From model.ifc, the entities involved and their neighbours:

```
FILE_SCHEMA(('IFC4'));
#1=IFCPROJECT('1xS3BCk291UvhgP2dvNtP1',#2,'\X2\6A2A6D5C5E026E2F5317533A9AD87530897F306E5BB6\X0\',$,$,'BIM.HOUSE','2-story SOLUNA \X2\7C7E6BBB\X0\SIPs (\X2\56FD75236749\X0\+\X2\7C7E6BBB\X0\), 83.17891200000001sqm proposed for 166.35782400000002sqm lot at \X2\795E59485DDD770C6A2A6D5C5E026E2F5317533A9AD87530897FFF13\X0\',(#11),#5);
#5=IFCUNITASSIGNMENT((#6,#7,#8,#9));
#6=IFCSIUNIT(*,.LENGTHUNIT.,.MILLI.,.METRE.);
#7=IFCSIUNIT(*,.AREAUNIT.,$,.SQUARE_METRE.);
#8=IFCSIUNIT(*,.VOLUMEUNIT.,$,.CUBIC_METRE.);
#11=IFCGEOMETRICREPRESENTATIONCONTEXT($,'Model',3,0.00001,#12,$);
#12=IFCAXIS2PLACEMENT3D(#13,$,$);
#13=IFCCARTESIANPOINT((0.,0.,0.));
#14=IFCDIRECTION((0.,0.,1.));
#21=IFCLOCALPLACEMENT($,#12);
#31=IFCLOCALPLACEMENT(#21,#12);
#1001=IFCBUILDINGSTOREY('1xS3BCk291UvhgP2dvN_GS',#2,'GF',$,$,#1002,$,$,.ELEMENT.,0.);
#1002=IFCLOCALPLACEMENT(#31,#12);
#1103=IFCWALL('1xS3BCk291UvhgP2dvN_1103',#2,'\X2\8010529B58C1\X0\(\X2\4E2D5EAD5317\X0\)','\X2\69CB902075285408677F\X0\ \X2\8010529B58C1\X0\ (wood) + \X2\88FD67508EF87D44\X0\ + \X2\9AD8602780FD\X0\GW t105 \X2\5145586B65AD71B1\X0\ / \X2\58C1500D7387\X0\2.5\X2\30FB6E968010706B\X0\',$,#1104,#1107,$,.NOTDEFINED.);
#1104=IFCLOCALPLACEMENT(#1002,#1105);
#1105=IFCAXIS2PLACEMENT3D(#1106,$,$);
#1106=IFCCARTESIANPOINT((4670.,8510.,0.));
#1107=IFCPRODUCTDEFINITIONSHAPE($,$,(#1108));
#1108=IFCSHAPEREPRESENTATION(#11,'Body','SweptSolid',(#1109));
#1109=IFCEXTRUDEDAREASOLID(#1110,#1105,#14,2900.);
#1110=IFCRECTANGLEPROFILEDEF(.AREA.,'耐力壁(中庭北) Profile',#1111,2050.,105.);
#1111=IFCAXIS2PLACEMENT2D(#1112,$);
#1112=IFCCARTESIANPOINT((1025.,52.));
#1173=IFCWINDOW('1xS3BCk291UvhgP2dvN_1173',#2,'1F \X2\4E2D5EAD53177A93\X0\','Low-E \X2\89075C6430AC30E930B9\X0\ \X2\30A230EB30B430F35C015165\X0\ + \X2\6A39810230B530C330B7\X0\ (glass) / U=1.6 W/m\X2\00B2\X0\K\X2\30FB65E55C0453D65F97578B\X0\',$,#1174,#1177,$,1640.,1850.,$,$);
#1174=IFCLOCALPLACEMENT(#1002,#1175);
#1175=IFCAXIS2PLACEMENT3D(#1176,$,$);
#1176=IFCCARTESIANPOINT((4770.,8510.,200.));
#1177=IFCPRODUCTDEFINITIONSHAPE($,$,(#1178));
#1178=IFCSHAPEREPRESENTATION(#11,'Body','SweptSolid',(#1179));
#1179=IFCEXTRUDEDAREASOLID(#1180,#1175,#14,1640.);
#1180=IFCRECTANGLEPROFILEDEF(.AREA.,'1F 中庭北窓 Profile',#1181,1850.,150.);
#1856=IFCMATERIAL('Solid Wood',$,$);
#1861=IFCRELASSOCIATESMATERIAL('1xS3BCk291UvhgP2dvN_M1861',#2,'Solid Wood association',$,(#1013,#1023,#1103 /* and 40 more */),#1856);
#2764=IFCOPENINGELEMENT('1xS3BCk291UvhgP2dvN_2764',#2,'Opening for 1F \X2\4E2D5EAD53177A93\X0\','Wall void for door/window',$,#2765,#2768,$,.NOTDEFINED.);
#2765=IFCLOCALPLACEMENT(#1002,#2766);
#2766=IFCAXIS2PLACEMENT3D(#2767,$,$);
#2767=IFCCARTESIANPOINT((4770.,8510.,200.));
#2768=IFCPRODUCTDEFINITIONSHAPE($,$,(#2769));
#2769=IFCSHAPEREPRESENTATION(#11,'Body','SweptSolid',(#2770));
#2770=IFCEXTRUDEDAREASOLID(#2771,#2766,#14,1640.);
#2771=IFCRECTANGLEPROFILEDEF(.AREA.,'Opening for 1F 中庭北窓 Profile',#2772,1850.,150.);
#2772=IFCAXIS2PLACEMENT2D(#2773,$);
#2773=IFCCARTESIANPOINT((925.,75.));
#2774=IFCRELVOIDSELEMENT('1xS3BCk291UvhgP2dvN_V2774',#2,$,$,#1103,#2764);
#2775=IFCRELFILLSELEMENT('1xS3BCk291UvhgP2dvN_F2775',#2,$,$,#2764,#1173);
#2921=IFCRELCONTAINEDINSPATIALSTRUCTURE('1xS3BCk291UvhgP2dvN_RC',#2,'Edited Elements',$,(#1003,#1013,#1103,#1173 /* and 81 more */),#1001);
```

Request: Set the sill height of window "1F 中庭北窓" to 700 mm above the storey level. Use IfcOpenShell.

```python
import numpy as np
import ifcopenshell
import ifcopenshell.api.geometry
import ifcopenshell.geom
import ifcopenshell.util.element
import ifcopenshell.util.placement
import ifcopenshell.util.shape
import ifcopenshell.util.unit

model = ifcopenshell.open("model.ifc")
unit_scale = ifcopenshell.util.unit.calculate_unit_scale(model)

window = model.by_guid("1xS3BCk291UvhgP2dvN_1173")
opening = window.FillsVoids[0].RelatingOpeningElement
storey = ifcopenshell.util.element.get_container(window, ifc_class="IfcBuildingStorey")
level = ifcopenshell.util.placement.get_local_placement(storey.ObjectPlacement)[2, 3]

# The opening's origin need not be at the sill, so measure its lowest point.
shape = ifcopenshell.geom.create_shape(ifcopenshell.geom.settings(), opening)
bottom = ifcopenshell.util.shape.get_shape_bottom_elevation(shape, shape.geometry) / unit_scale
dz = level + 700.0 - bottom

shift = np.array([0.0, 0.0, dz])
# The window is not placed relative to its opening, so move both.
for product in (opening, window):
    matrix = ifcopenshell.util.placement.get_local_placement(product.ObjectPlacement)
    matrix[:3, 3] += shift
    ifcopenshell.api.geometry.edit_object_placement(model, product=product, matrix=matrix, is_si=False)

print(f"moved by {dz * unit_scale:+.3f} m")

model.write("model-out.ifc")
```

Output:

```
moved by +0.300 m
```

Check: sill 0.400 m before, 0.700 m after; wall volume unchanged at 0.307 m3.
